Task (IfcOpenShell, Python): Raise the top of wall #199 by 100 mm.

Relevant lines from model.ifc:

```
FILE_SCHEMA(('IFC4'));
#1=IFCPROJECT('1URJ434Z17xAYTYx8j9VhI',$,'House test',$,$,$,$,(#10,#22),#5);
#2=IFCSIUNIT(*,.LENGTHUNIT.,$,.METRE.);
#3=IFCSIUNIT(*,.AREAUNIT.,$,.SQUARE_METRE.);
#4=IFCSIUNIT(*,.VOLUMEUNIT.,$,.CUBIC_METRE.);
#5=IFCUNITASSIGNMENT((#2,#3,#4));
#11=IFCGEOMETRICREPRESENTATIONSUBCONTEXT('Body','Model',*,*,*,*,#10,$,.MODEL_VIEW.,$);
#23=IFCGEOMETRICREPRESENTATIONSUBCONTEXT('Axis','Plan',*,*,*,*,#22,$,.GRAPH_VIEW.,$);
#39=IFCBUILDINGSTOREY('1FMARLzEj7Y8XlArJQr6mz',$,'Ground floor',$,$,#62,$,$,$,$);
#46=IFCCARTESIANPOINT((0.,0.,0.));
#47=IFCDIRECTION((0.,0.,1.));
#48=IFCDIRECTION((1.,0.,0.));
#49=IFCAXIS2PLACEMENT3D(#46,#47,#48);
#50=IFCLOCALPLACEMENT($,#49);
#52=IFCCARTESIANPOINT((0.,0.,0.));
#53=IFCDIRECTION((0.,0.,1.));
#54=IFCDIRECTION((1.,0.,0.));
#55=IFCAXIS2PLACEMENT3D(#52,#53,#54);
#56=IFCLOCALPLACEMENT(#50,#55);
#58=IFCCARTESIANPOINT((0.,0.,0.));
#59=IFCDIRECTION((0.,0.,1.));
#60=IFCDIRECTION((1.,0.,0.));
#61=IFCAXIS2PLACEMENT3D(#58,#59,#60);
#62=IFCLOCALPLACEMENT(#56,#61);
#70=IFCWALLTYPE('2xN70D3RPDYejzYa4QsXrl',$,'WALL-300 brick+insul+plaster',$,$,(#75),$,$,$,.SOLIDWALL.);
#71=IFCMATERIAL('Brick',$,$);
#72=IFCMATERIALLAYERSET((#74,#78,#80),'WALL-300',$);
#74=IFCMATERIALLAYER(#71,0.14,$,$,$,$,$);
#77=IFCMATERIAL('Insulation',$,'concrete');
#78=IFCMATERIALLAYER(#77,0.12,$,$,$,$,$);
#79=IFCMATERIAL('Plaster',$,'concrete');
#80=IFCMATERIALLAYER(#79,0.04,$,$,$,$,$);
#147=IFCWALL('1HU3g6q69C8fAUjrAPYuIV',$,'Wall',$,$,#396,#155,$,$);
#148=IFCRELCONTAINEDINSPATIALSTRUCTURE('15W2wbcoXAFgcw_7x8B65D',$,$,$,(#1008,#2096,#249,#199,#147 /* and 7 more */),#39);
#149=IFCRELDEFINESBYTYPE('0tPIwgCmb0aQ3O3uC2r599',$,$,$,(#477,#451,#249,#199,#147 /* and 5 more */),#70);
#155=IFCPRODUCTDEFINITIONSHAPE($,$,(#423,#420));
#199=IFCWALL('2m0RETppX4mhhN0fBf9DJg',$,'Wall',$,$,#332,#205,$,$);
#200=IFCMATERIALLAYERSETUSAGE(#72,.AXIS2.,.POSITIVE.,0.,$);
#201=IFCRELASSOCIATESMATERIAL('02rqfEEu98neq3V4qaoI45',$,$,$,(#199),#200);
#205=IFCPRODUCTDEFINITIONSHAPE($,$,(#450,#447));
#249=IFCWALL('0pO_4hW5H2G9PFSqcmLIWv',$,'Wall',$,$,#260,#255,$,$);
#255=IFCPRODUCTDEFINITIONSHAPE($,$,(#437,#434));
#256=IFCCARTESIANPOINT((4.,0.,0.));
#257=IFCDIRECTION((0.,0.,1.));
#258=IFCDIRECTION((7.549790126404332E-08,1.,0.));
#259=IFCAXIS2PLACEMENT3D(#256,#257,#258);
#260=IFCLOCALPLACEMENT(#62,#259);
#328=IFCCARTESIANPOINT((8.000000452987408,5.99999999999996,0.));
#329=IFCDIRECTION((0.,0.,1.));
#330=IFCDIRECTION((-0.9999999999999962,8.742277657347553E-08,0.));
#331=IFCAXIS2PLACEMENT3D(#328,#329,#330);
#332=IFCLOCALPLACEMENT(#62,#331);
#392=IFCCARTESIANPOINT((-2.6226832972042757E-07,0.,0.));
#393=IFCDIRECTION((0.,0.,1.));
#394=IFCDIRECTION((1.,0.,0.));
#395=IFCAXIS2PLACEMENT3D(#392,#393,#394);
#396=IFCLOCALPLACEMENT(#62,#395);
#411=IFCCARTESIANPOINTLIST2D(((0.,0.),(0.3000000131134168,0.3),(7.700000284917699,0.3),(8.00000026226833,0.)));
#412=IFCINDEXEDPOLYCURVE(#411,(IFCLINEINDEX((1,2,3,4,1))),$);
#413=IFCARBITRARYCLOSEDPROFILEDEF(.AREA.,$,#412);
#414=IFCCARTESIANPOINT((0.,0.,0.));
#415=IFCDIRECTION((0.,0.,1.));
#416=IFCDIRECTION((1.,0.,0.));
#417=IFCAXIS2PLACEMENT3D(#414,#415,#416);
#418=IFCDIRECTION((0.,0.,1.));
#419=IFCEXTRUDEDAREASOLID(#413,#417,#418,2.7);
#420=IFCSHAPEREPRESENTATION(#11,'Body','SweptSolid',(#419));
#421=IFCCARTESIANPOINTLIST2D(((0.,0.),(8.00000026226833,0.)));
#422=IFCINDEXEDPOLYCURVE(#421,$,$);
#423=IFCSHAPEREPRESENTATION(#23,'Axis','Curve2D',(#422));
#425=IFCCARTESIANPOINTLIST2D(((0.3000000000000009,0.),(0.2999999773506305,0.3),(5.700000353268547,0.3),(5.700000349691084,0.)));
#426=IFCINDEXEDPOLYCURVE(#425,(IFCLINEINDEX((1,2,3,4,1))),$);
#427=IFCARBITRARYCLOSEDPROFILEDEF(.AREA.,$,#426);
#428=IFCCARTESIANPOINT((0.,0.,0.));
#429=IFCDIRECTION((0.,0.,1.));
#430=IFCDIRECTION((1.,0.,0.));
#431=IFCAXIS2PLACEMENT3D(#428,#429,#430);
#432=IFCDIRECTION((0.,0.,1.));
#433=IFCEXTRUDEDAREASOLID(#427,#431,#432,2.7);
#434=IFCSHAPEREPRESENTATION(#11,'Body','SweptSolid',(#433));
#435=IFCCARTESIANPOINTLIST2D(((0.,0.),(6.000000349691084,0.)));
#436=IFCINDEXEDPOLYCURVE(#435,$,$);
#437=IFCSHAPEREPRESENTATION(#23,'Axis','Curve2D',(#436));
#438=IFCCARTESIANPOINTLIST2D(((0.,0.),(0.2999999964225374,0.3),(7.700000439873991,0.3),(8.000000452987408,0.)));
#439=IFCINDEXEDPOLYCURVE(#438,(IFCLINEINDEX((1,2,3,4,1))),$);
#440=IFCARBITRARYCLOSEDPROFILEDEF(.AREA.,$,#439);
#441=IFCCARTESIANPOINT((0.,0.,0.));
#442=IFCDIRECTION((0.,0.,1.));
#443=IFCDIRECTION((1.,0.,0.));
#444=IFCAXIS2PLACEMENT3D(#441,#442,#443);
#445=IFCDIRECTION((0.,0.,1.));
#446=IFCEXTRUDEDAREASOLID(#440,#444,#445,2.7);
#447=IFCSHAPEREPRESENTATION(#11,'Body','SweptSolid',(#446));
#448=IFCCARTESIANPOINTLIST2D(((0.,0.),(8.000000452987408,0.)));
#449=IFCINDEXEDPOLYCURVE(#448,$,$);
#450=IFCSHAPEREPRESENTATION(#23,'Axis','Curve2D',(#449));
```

```python
import ifcopenshell
import ifcopenshell.geom
import ifcopenshell.util.representation
import ifcopenshell.util.shape

model = ifcopenshell.open("model.ifc")
settings = ifcopenshell.geom.settings()


def volume(element):
    """Net volume in cubic metres, openings subtracted."""
    shape = ifcopenshell.geom.create_shape(settings, element)
    return ifcopenshell.util.shape.get_volume(shape.geometry)


wall = model.by_id(199)
before = volume(wall)

body = ifcopenshell.util.representation.get_representation(wall, "Model", "Body")
solid = body.Items[0]
old_height = solid.Depth
solid.Depth += 0.1
after = volume(wall)

print(f"height {old_height:g} -> {solid.Depth:g}, volume {before:.3f} -> {after:.3f} m3")

model.write("model_edited.ifc")
```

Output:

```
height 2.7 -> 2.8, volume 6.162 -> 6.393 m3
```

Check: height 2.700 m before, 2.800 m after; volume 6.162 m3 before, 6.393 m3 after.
